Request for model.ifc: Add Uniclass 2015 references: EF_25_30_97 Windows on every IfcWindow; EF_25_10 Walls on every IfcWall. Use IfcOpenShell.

First a look at what the model holds.

```python
import ifcopenshell

model = ifcopenshell.open("model.ifc")
print(model.schema)
print("classifications:", [c.Name for c in model.by_type("IfcClassification")])
for ifc_class in ("IfcDoor", "IfcRoof", "IfcStair", "IfcWall", "IfcWindow"):
    print(ifc_class, len(model.by_type(ifc_class)))
```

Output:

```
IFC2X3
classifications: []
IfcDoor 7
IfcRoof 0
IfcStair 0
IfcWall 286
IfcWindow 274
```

```python
import ifcopenshell
import ifcopenshell.api.classification

model = ifcopenshell.open("model.ifc")

# IFC2X3 requires Source and Edition and has no link from the project to the system.
system = model.create_entity("IfcClassification", Source="NBS", Edition="2015", Name="Uniclass 2015")

codes = {
    "IfcWindow": ("EF_25_30_97", "Windows"),
    "IfcWall": ("EF_25_10", "Walls"),
}
for ifc_class, (code, name) in codes.items():
    products = model.by_type(ifc_class)
    ifcopenshell.api.classification.add_reference(
        model, products=products, classification=system, identification=code, name=name
    )
    print(code, len(products))

model.write("model_rev.ifc")
```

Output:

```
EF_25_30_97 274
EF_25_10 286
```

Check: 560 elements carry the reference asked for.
